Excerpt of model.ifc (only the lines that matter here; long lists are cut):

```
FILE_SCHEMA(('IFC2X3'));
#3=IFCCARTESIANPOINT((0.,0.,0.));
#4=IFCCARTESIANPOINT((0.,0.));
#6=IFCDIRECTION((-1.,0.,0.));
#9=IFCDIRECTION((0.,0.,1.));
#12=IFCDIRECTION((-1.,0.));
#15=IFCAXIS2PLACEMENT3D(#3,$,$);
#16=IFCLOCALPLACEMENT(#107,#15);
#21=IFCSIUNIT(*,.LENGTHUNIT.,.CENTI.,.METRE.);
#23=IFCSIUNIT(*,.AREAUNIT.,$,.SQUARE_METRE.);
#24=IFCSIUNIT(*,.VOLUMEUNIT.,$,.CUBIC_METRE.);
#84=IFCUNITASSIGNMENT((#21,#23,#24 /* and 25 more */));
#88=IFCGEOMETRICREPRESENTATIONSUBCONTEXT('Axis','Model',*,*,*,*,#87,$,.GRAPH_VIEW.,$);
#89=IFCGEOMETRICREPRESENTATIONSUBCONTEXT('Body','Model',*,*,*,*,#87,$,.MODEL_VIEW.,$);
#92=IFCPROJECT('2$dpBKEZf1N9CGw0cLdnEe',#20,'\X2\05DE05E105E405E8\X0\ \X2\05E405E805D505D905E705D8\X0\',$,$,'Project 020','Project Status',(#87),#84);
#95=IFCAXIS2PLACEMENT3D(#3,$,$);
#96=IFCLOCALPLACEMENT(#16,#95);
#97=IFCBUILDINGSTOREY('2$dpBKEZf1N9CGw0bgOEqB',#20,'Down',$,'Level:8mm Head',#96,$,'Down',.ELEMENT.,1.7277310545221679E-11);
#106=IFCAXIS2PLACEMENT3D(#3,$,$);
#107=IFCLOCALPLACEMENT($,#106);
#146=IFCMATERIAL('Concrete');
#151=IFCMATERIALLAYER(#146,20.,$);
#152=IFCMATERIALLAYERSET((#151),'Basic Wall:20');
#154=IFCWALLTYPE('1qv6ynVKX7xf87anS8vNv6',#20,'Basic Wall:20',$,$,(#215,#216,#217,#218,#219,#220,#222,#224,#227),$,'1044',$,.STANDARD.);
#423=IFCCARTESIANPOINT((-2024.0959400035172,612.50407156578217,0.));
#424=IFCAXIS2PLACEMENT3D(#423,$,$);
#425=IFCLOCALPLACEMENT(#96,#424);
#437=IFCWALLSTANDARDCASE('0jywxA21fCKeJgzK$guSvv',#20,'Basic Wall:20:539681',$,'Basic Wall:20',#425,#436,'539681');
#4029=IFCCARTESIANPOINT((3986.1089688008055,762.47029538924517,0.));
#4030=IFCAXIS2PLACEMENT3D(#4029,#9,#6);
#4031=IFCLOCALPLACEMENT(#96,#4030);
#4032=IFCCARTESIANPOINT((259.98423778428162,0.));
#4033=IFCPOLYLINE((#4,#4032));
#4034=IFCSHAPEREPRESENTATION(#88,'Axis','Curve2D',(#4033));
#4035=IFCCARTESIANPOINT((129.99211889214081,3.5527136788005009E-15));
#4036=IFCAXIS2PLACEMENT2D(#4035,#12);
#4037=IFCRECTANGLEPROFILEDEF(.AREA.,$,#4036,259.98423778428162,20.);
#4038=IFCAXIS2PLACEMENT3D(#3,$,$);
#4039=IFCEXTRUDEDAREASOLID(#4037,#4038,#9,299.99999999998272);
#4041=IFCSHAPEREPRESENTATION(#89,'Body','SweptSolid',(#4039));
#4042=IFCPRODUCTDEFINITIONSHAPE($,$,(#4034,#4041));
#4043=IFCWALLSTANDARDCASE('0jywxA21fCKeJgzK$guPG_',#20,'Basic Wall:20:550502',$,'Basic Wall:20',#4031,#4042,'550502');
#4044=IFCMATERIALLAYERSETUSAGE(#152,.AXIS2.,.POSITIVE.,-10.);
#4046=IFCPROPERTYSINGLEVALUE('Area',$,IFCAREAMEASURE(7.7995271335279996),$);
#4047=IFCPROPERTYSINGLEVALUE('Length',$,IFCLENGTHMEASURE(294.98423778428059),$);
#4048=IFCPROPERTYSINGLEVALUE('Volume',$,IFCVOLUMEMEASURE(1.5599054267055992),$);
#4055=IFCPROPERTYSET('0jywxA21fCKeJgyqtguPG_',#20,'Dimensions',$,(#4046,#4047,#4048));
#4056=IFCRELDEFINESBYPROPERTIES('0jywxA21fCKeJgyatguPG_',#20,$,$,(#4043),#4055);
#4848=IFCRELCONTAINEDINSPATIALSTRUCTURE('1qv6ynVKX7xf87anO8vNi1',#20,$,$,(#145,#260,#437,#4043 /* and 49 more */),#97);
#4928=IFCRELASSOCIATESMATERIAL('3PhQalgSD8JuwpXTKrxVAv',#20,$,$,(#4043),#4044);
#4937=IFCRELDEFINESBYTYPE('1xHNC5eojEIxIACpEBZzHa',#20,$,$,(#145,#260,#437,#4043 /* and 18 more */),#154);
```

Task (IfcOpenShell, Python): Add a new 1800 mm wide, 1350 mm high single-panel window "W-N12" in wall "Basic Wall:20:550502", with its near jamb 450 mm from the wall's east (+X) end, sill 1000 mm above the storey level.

```python
import numpy as np
import ifcopenshell
import ifcopenshell.api.feature
import ifcopenshell.api.geometry
import ifcopenshell.api.pset
import ifcopenshell.api.root
import ifcopenshell.api.spatial
import ifcopenshell.api.type
import ifcopenshell.geom
import ifcopenshell.util.element
import ifcopenshell.util.placement
import ifcopenshell.util.representation
import ifcopenshell.util.shape
import ifcopenshell.util.unit

model = ifcopenshell.open("model.ifc")
unit_scale = ifcopenshell.util.unit.calculate_unit_scale(model)
area_scale = ifcopenshell.util.unit.calculate_unit_scale(model, "AREAUNIT")
volume_scale = ifcopenshell.util.unit.calculate_unit_scale(model, "VOLUMEUNIT")
settings = ifcopenshell.geom.settings()


def volume(element):
    """Net volume in cubic metres, openings subtracted."""
    shape = ifcopenshell.geom.create_shape(settings, element)
    return ifcopenshell.util.shape.get_volume(shape.geometry)


wall = model.by_guid("0jywxA21fCKeJgzK$guPG_")
storey = ifcopenshell.util.element.get_container(wall, ifc_class="IfcBuildingStorey")
context = ifcopenshell.util.representation.get_context(model, "Model", "Body", "MODEL_VIEW")
before = volume(wall)

width, height, from_end, sill = 1.8, 1.35, 0.45, 1  # metres

# The wall runs along its own X axis, and the end named is its -X end.
wall_shape = ifcopenshell.geom.create_shape(settings, wall)
x, y, z = ifcopenshell.util.shape.get_vertices(wall_shape.geometry).T
start = x.min() + from_end
face, thickness = float(y.min()), float(y.max() - y.min())
wall_matrix = ifcopenshell.util.placement.get_local_placement(wall.ObjectPlacement)
level = ifcopenshell.util.placement.get_local_placement(storey.ObjectPlacement)[2, 3]


def in_wall(x, y):
    """Placement at x, y metres in the wall's axes, at sill height."""
    matrix = wall_matrix.copy()
    matrix[:, 3] = wall_matrix @ np.array([x / unit_scale, y / unit_scale, 0.0, 1.0])
    matrix[2, 3] = level + sill / unit_scale
    return matrix


# Opening: a box that overshoots both wall faces by 50 mm.
opening = ifcopenshell.api.root.create_entity(model, ifc_class="IfcOpeningElement")
box = ifcopenshell.api.geometry.add_wall_representation(
    model, context=context, length=width, height=height, thickness=thickness + 0.1
)
ifcopenshell.api.geometry.assign_representation(model, product=opening, representation=box)
ifcopenshell.api.geometry.edit_object_placement(model, product=opening, matrix=in_wall(start, face - 0.05), is_si=False)
ifcopenshell.api.feature.add_feature(model, feature=opening, element=wall)

window = ifcopenshell.api.root.create_entity(model, ifc_class="IfcWindow", name="W-N12")
window.OverallWidth, window.OverallHeight = width / unit_scale, height / unit_scale
body = ifcopenshell.api.geometry.add_window_representation(
    model,
    context=context,
    overall_width=window.OverallWidth,
    overall_height=window.OverallHeight,
    partition_type="SINGLE_PANEL",
)
ifcopenshell.api.geometry.assign_representation(model, product=window, representation=body)
ifcopenshell.api.spatial.assign_container(model, products=[window], relating_structure=storey)
fills = ifcopenshell.api.feature.add_filling(model, opening=opening, element=window)
fills.OwnerHistory = window.OwnerHistory  # required in IFC2X3

# IFC2X3 keeps the operation on the window style.
style = ifcopenshell.api.root.create_entity(model, ifc_class="IfcWindowStyle", name="W-N12")
style.OperationType, style.ConstructionType = "SINGLE_PANEL", "NOTDEFINED"
style.ParameterTakesPrecedence = style.Sizeable = False
ifcopenshell.api.type.assign_type(model, related_objects=[window], relating_type=style)

# Centre the window in the wall's thickness.
ifcopenshell.api.geometry.edit_object_placement(model, product=window, matrix=in_wall(start, face), is_si=False)
window_shape = ifcopenshell.geom.create_shape(settings, window)
depth = ifcopenshell.util.shape.get_vertices(window_shape.geometry)[:, 1]
offset = face + thickness / 2 - (depth.min() + depth.max()) / 2
ifcopenshell.api.geometry.edit_object_placement(model, product=window, matrix=in_wall(start, offset), is_si=False)

after = volume(wall)

# Update the wall's stored quantities.
pset = model.by_id(ifcopenshell.util.element.get_pset(wall, "Dimensions", should_inherit=False)["id"])
ifcopenshell.api.pset.edit_pset(model, pset=pset, properties={
    "Area": model.create_entity("IfcAreaMeasure", after / thickness / area_scale),
    "Volume": model.create_entity("IfcVolumeMeasure", after / volume_scale),
})

print(f"wall volume {before:.3f} -> {after:.3f} m3")

model.write("model_v2.ifc")
```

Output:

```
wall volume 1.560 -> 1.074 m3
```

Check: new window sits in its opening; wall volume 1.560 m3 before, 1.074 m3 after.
